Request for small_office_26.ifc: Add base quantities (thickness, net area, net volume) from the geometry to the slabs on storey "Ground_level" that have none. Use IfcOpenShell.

First a look at what the model holds.

```python
import ifcopenshell
import ifcopenshell.util.element
import ifcopenshell.util.unit

model = ifcopenshell.open("small_office_26.ifc")
print(model.schema)
for unit_type in ("LENGTHUNIT", "AREAUNIT", "VOLUMEUNIT"):
    print(unit_type, ifcopenshell.util.unit.calculate_unit_scale(model, unit_type))
storey = next(s for s in model.by_type("IfcBuildingStorey") if s.Name == "Ground_level")
slabs = [e for e in ifcopenshell.util.element.get_decomposition(storey) if e.is_a("IfcSlab")]
for e in sorted(slabs, key=lambda e: e.id()):
    print(e.id(), e.is_a(), e.Name, list(ifcopenshell.util.element.get_psets(e, qtos_only=True)), sep=" | ")
```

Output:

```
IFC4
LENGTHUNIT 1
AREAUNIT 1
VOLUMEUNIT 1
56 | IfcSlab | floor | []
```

```python
import ifcopenshell
import ifcopenshell.api.pset
import ifcopenshell.geom
import ifcopenshell.util.element
import ifcopenshell.util.shape
import ifcopenshell.util.unit

model = ifcopenshell.open("small_office_26.ifc")
unit_scale = ifcopenshell.util.unit.calculate_unit_scale(model)
area_scale = ifcopenshell.util.unit.calculate_unit_scale(model, "AREAUNIT")
volume_scale = ifcopenshell.util.unit.calculate_unit_scale(model, "VOLUMEUNIT")
settings = ifcopenshell.geom.settings()

storey = next(s for s in model.by_type("IfcBuildingStorey") if s.Name == "Ground_level")
slabs = [e for e in ifcopenshell.util.element.get_decomposition(storey) if e.is_a("IfcSlab")]

for e in sorted(slabs, key=lambda e: e.id()):
    if ifcopenshell.util.element.get_psets(e, qtos_only=True, should_inherit=False):
        continue
    # Geometry comes back in metres, in the element's own axes.
    shape = ifcopenshell.geom.create_shape(settings, e)
    values = {
        "Width": ifcopenshell.util.shape.get_z(shape.geometry) / unit_scale,
        "NetArea": ifcopenshell.util.shape.get_footprint_area(shape.geometry) / area_scale,
        "NetVolume": ifcopenshell.util.shape.get_volume(shape.geometry) / volume_scale,
    }
    qto = ifcopenshell.api.pset.add_qto(model, product=e, name="Qto_SlabBaseQuantities")
    ifcopenshell.api.pset.edit_qto(model, qto=qto, properties=values)
    print(e.id(), {k: round(v, 3) for k, v in values.items()})

model.write("small_office_26_rev.ifc")
```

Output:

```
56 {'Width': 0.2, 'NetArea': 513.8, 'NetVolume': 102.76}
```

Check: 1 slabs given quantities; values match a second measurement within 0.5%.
